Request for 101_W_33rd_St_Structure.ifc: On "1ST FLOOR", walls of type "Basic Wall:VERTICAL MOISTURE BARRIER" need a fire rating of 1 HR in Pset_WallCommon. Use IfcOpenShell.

First a look at what the model holds.

```python
import ifcopenshell
import ifcopenshell.util.element

model = ifcopenshell.open("101_W_33rd_St_Structure.ifc")
print(model.schema)
storey = next(s for s in model.by_type("IfcBuildingStorey") if s.Name == "1ST FLOOR")
walls = [e for e in ifcopenshell.util.element.get_decomposition(storey) if e.is_a("IfcWall")]
seen = {}
for e in walls:
    element_type = ifcopenshell.util.element.get_type(e)
    key = (element_type.Name if element_type != e and element_type else None, ifcopenshell.util.element.get_pset(e, "Pset_WallCommon", "FireRating"))
    seen[key] = seen.get(key, 0) + 1
for (name, value), count in sorted(seen.items(), key=str):
    print(count, "x", name, "|", value)
```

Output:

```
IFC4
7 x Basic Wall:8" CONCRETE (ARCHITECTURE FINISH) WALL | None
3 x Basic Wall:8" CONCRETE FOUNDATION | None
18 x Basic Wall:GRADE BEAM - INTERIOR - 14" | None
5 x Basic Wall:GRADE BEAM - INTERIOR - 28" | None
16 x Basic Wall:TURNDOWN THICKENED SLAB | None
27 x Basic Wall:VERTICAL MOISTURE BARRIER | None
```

```python
import ifcopenshell
import ifcopenshell.api.pset
import ifcopenshell.util.element

model = ifcopenshell.open("101_W_33rd_St_Structure.ifc")

storey = next(s for s in model.by_type("IfcBuildingStorey") if s.Name == "1ST FLOOR")
walls = [e for e in ifcopenshell.util.element.get_decomposition(storey) if e.is_a("IfcWall")]

count = 0
for e in walls:
    element_type = ifcopenshell.util.element.get_type(e)
    if element_type in (None, e) or element_type.Name != "Basic Wall:VERTICAL MOISTURE BARRIER":
        continue
    # add_pset returns the element's existing set when there is one.
    pset = ifcopenshell.api.pset.add_pset(model, product=e, name="Pset_WallCommon")
    ifcopenshell.api.pset.edit_pset(model, pset=pset, properties={"FireRating": "1 HR"})
    count += 1

print(count, "walls updated")

model.write("101_W_33rd_St_Structure_rev.ifc")
```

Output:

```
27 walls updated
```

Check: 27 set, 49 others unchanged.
